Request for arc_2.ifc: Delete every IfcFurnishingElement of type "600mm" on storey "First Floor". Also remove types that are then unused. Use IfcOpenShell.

First a look at what the model holds.

```python
import ifcopenshell
import ifcopenshell.util.element

model = ifcopenshell.open("arc_2.ifc")
print(model.schema)
storey = next(s for s in model.by_type("IfcBuildingStorey") if s.Name == "First Floor")
furniture = [e for e in ifcopenshell.util.element.get_decomposition(storey) if e.is_a("IfcFurnishingElement")]
seen = {}
for e in furniture:
    element_type = ifcopenshell.util.element.get_type(e)
    name = element_type.Name if element_type not in (None, e) else None
    seen[name] = seen.get(name, 0) + 1
for name, count in sorted(seen.items(), key=str):
    print(count, "x", name)
```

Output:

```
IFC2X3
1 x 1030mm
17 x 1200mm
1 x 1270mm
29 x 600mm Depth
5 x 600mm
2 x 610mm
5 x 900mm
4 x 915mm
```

```python
import ifcopenshell
import ifcopenshell.api.root
import ifcopenshell.util.element

model = ifcopenshell.open("arc_2.ifc")

storey = next(s for s in model.by_type("IfcBuildingStorey") if s.Name == "First Floor")
furniture = [e for e in ifcopenshell.util.element.get_decomposition(storey) if e.is_a("IfcFurnishingElement")]
targets = [e for e in furniture if (t := ifcopenshell.util.element.get_type(e)) not in (None, e) and t.Name == "600mm"]
types = {ifcopenshell.util.element.get_type(e) for e in targets} - {None, *targets}

for e in targets:
    ifcopenshell.api.root.remove_product(model, product=e)
print(len(targets), "removed")

unused = [t for t in types if not ifcopenshell.util.element.get_types(t)]
for t in unused:
    ifcopenshell.api.root.remove_product(model, product=t)
print(len(unused), "unused types removed")

model.write("arc_2_rev.ifc")
```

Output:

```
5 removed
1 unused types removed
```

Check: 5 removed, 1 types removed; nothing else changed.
